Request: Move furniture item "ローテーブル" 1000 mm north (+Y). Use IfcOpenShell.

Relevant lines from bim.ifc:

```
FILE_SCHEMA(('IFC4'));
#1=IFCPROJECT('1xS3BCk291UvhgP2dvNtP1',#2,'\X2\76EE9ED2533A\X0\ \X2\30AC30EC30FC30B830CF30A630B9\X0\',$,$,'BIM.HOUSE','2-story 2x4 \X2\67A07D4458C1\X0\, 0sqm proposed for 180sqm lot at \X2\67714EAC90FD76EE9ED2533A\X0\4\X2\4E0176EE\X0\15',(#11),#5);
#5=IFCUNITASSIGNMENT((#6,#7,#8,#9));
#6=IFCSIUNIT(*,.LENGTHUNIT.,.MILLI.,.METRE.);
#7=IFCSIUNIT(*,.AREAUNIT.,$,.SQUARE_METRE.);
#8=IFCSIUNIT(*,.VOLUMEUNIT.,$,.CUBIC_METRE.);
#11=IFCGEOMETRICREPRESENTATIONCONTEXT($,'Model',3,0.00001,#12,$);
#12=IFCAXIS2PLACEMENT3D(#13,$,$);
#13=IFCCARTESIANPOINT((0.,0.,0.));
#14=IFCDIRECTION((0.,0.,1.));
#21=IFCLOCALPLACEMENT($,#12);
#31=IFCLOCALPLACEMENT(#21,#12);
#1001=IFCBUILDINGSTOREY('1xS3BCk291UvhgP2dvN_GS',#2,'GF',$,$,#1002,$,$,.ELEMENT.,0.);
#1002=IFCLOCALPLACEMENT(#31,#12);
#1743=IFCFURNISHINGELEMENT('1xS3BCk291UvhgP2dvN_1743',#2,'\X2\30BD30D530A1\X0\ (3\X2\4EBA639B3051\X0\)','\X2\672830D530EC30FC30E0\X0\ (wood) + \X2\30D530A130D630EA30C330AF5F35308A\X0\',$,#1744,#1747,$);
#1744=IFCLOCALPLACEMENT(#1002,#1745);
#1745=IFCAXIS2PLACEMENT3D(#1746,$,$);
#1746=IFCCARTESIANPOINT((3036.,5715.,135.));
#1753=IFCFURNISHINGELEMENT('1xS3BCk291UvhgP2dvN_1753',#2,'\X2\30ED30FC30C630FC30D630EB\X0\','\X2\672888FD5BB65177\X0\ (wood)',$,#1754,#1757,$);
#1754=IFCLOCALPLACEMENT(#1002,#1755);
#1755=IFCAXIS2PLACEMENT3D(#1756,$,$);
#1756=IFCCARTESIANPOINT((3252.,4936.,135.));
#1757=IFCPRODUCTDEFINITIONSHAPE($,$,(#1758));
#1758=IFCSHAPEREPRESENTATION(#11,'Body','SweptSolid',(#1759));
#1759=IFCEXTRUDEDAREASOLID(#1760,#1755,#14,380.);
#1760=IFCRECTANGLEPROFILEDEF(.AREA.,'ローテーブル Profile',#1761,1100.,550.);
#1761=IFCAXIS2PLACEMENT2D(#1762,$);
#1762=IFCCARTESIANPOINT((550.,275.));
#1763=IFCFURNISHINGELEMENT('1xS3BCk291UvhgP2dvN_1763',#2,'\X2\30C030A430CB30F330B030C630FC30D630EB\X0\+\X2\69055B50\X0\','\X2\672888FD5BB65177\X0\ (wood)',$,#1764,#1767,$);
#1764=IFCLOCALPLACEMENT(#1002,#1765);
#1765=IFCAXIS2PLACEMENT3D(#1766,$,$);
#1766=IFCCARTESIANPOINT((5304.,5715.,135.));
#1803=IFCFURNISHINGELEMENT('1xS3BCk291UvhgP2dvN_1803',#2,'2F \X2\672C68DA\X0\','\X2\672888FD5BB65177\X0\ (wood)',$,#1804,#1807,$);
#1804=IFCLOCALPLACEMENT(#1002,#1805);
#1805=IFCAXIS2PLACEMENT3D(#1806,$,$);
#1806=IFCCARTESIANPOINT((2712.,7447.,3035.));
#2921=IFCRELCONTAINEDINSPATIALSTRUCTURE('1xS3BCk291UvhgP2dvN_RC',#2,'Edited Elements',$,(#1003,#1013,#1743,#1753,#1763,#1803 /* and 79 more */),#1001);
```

```python
import ifcopenshell
import ifcopenshell.api.geometry
import ifcopenshell.util.placement

model = ifcopenshell.open("bim.ifc")

item = model.by_guid("1xS3BCk291UvhgP2dvN_1753")
matrix = ifcopenshell.util.placement.get_local_placement(item.ObjectPlacement)
matrix[1, 3] += 1000.0
ifcopenshell.api.geometry.edit_object_placement(model, product=item, matrix=matrix, is_si=False)

print(ifcopenshell.util.placement.get_local_placement(item.ObjectPlacement).round(3) + 0.0)

model.write("bim_edited.ifc")
```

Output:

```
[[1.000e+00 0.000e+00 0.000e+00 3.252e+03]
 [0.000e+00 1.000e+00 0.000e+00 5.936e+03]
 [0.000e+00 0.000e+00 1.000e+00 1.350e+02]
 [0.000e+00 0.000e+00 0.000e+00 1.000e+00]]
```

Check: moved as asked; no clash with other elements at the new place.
